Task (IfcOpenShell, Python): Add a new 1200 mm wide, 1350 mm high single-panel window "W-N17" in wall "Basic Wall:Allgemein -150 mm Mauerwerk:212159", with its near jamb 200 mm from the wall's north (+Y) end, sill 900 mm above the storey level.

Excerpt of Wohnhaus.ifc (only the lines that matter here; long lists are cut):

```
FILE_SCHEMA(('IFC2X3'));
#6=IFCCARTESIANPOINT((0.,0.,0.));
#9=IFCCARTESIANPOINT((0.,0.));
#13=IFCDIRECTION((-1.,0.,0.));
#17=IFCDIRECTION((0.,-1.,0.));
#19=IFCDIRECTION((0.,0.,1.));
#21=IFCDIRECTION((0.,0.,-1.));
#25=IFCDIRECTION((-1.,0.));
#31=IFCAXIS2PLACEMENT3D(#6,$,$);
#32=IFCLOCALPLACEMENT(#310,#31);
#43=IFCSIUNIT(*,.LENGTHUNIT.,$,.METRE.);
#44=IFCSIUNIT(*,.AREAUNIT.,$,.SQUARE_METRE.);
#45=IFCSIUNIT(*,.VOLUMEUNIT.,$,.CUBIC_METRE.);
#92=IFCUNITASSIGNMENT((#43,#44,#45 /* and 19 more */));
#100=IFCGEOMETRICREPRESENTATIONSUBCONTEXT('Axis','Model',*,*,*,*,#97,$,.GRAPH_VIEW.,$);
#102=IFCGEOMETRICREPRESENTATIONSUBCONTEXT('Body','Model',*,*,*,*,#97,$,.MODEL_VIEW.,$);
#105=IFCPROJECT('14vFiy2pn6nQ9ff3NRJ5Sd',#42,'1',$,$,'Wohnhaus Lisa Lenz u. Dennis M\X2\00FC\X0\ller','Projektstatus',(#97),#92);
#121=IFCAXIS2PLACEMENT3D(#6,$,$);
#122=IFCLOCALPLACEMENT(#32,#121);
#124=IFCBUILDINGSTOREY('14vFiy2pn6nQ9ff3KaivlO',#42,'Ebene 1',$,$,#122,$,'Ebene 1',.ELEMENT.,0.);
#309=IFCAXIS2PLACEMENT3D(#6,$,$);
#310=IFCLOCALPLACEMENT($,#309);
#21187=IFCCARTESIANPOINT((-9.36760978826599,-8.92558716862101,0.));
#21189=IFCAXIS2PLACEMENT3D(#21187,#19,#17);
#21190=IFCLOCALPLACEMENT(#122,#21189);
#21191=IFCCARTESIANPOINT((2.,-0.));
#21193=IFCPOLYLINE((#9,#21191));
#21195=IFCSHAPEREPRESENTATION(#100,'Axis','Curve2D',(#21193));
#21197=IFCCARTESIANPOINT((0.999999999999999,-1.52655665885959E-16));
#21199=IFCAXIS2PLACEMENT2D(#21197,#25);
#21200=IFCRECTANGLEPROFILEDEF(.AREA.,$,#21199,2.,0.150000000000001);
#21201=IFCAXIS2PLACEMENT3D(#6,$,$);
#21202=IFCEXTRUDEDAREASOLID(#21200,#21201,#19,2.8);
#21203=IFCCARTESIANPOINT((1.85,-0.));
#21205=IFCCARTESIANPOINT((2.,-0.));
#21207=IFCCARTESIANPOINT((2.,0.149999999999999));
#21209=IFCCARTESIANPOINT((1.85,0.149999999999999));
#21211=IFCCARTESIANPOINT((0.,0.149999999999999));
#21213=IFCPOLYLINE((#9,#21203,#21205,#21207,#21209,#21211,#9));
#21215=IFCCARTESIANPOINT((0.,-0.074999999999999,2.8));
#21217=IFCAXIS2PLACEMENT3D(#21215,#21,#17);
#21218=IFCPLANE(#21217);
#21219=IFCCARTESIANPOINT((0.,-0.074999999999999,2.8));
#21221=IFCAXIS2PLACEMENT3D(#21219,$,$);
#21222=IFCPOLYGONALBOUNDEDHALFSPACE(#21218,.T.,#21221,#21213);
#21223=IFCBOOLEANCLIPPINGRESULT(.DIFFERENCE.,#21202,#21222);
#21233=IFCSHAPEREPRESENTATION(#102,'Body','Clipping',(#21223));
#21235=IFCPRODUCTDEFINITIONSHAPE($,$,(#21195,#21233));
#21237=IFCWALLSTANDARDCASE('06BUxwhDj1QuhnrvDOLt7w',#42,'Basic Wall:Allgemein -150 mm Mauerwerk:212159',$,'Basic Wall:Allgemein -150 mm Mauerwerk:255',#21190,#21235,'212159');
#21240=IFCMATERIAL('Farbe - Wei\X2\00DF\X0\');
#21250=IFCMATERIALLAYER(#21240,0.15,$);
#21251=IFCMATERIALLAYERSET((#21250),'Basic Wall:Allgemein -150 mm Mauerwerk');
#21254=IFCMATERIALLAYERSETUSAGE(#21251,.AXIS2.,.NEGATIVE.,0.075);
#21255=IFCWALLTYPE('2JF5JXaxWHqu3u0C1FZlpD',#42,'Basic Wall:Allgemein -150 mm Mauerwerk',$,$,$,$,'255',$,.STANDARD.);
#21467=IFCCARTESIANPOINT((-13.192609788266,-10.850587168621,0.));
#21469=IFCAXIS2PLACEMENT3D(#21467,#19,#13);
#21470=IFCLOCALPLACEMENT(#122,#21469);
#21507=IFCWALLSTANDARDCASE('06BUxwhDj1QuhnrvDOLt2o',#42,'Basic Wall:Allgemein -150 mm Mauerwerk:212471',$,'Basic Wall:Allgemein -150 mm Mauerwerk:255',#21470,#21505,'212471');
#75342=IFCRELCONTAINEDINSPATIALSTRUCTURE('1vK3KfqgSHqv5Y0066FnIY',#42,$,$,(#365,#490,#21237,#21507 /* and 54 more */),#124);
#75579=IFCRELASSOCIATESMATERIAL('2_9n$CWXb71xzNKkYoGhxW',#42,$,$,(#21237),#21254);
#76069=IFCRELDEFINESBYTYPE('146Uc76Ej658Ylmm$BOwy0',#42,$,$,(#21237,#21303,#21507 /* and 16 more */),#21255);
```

```python
import numpy as np
import ifcopenshell
import ifcopenshell.api.feature
import ifcopenshell.api.geometry
import ifcopenshell.api.root
import ifcopenshell.api.spatial
import ifcopenshell.api.type
import ifcopenshell.geom
import ifcopenshell.util.element
import ifcopenshell.util.placement
import ifcopenshell.util.representation
import ifcopenshell.util.shape
import ifcopenshell.util.unit

model = ifcopenshell.open("Wohnhaus.ifc")
unit_scale = ifcopenshell.util.unit.calculate_unit_scale(model)
settings = ifcopenshell.geom.settings()


def volume(element):
    """Net volume in cubic metres, openings subtracted."""
    shape = ifcopenshell.geom.create_shape(settings, element)
    return ifcopenshell.util.shape.get_volume(shape.geometry)


wall = model.by_guid("06BUxwhDj1QuhnrvDOLt7w")
storey = ifcopenshell.util.element.get_container(wall, ifc_class="IfcBuildingStorey")
context = ifcopenshell.util.representation.get_context(model, "Model", "Body", "MODEL_VIEW")
before = volume(wall)

width, height, from_end, sill = 1.2, 1.35, 0.2, 0.9  # metres

# The wall runs along its own X axis, and the end named is its -X end.
wall_shape = ifcopenshell.geom.create_shape(settings, wall)
x, y, z = ifcopenshell.util.shape.get_vertices(wall_shape.geometry).T
start = x.min() + from_end
face, thickness = float(y.min()), float(y.max() - y.min())
wall_matrix = ifcopenshell.util.placement.get_local_placement(wall.ObjectPlacement)
level = ifcopenshell.util.placement.get_local_placement(storey.ObjectPlacement)[2, 3]


def in_wall(x, y):
    """Placement at x, y metres in the wall's axes, at sill height."""
    matrix = wall_matrix.copy()
    matrix[:, 3] = wall_matrix @ np.array([x / unit_scale, y / unit_scale, 0.0, 1.0])
    matrix[2, 3] = level + sill / unit_scale
    return matrix


# Opening: a box that overshoots both wall faces by 50 mm.
opening = ifcopenshell.api.root.create_entity(model, ifc_class="IfcOpeningElement")
box = ifcopenshell.api.geometry.add_wall_representation(
    model, context=context, length=width, height=height, thickness=thickness + 0.1
)
ifcopenshell.api.geometry.assign_representation(model, product=opening, representation=box)
ifcopenshell.api.geometry.edit_object_placement(model, product=opening, matrix=in_wall(start, face - 0.05), is_si=False)
ifcopenshell.api.feature.add_feature(model, feature=opening, element=wall)

window = ifcopenshell.api.root.create_entity(model, ifc_class="IfcWindow", name="W-N17")
window.OverallWidth, window.OverallHeight = width / unit_scale, height / unit_scale
body = ifcopenshell.api.geometry.add_window_representation(
    model,
    context=context,
    overall_width=window.OverallWidth,
    overall_height=window.OverallHeight,
    partition_type="SINGLE_PANEL",
)
ifcopenshell.api.geometry.assign_representation(model, product=window, representation=body)
ifcopenshell.api.spatial.assign_container(model, products=[window], relating_structure=storey)
fills = ifcopenshell.api.feature.add_filling(model, opening=opening, element=window)
fills.OwnerHistory = window.OwnerHistory  # required in IFC2X3

# IFC2X3 keeps the operation on the window style.
style = ifcopenshell.api.root.create_entity(model, ifc_class="IfcWindowStyle", name="W-N17")
style.OperationType, style.ConstructionType = "SINGLE_PANEL", "NOTDEFINED"
style.ParameterTakesPrecedence = style.Sizeable = False
ifcopenshell.api.type.assign_type(model, related_objects=[window], relating_type=style)

# Centre the window in the wall's thickness.
ifcopenshell.api.geometry.edit_object_placement(model, product=window, matrix=in_wall(start, face), is_si=False)
window_shape = ifcopenshell.geom.create_shape(settings, window)
depth = ifcopenshell.util.shape.get_vertices(window_shape.geometry)[:, 1]
offset = face + thickness / 2 - (depth.min() + depth.max()) / 2
ifcopenshell.api.geometry.edit_object_placement(model, product=window, matrix=in_wall(start, offset), is_si=False)

after = volume(wall)

print(f"wall volume {before:.3f} -> {after:.3f} m3")

model.write("Wohnhaus-out.ifc")
```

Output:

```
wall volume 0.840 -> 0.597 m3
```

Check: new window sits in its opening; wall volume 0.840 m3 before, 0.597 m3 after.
